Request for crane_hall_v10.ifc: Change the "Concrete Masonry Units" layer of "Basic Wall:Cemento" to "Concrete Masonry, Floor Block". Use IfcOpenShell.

First a look at what the model holds.

```python
import ifcopenshell
import ifcopenshell.util.element

model = ifcopenshell.open("crane_hall_v10.ifc")
print(model.schema)
for layer_set in model.by_type("IfcMaterialLayerSet"):
    if layer_set.LayerSetName == "Basic Wall:Cemento":
        for layer in layer_set.MaterialLayers:
            print(layer.id(), layer.Material and layer.Material.Name, layer.LayerThickness, sep=" | ")
        print(len(ifcopenshell.util.element.get_elements_by_material(model, layer_set)), "elements and types use it")
print(sorted(m.Name for m in model.by_type("IfcMaterial") if m.Name)[:60])
```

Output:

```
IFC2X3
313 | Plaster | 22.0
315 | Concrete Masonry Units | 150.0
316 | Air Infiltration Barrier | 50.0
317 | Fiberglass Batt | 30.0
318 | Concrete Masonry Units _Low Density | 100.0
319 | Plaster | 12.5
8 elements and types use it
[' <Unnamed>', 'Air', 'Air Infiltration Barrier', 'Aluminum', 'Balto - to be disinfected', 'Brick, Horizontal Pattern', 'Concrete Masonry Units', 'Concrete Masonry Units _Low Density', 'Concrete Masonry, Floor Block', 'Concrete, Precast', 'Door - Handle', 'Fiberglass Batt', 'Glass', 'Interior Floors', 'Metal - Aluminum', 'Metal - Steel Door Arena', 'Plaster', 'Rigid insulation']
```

```python
import ifcopenshell
import ifcopenshell.api.material

model = ifcopenshell.open("crane_hall_v10.ifc")

layer_set = next(s for s in model.by_type("IfcMaterialLayerSet") if s.LayerSetName == "Basic Wall:Cemento")
layer = next(l for l in layer_set.MaterialLayers if l.Material and l.Material.Name == "Concrete Masonry Units")
material = next(m for m in model.by_type("IfcMaterial") if m.Name == "Concrete Masonry, Floor Block")

# Point this one layer at the other material; renaming the old one would change it everywhere.
ifcopenshell.api.material.edit_layer(model, layer=layer, attributes={}, material=material)

print([l.Material.Name if l.Material else None for l in layer_set.MaterialLayers])

model.write("crane_hall_v10_edited.ifc")
```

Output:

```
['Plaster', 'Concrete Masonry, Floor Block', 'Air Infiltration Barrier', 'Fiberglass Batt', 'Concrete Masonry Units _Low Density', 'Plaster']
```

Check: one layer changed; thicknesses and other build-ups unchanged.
